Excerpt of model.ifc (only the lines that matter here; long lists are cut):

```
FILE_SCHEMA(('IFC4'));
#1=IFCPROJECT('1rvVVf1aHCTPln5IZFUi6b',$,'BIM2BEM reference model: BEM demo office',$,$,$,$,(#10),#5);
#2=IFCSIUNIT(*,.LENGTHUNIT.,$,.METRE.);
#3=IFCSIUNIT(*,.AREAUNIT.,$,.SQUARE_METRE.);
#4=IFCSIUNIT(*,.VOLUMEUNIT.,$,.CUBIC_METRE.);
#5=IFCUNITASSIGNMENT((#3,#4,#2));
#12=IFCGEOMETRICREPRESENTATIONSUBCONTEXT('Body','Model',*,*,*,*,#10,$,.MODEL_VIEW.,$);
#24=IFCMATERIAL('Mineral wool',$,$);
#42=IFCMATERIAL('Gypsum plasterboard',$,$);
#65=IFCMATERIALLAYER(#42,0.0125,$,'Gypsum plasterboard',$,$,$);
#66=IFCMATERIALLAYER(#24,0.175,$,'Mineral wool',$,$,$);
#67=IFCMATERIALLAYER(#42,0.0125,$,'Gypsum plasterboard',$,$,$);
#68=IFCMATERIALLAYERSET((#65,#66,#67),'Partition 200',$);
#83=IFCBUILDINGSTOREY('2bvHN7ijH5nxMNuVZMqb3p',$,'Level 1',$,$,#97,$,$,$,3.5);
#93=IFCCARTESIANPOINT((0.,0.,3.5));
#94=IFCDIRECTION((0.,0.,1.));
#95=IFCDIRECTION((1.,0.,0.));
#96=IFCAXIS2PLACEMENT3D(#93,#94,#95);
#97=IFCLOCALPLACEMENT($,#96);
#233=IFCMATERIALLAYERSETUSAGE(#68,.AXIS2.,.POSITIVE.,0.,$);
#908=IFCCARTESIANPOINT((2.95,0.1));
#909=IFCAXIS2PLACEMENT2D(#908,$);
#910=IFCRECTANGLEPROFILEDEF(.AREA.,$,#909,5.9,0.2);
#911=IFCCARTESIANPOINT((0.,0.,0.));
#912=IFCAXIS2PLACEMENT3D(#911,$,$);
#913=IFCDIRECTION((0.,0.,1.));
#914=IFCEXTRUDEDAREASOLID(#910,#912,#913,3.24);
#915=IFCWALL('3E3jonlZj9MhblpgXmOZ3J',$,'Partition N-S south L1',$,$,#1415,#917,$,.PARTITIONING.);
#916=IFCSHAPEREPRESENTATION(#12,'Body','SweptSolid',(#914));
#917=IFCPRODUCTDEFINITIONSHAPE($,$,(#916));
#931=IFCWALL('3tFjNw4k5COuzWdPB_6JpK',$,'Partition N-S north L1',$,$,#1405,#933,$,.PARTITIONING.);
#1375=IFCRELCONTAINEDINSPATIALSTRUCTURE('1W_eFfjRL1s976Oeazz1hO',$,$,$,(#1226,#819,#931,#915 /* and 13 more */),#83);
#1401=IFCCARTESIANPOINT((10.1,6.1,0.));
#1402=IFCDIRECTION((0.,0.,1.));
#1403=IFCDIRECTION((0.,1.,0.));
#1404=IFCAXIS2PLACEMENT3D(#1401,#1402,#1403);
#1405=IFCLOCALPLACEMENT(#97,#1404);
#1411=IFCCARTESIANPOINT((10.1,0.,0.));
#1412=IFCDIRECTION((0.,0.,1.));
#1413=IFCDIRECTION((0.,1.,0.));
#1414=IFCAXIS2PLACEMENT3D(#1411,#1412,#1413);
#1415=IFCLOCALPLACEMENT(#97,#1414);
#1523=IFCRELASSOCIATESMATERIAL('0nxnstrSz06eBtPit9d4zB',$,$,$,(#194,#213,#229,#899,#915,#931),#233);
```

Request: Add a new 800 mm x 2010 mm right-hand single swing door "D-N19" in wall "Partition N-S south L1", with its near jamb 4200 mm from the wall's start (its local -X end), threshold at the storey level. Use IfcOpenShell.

```python
import numpy as np
import ifcopenshell
import ifcopenshell.api.feature
import ifcopenshell.api.geometry
import ifcopenshell.api.root
import ifcopenshell.api.spatial
import ifcopenshell.geom
import ifcopenshell.util.element
import ifcopenshell.util.placement
import ifcopenshell.util.representation
import ifcopenshell.util.shape
import ifcopenshell.util.unit

model = ifcopenshell.open("model.ifc")
unit_scale = ifcopenshell.util.unit.calculate_unit_scale(model)
settings = ifcopenshell.geom.settings()


def volume(element):
    """Net volume in cubic metres, openings subtracted."""
    shape = ifcopenshell.geom.create_shape(settings, element)
    return ifcopenshell.util.shape.get_volume(shape.geometry)


wall = model.by_guid("3E3jonlZj9MhblpgXmOZ3J")
storey = ifcopenshell.util.element.get_container(wall, ifc_class="IfcBuildingStorey")
context = ifcopenshell.util.representation.get_context(model, "Model", "Body", "MODEL_VIEW")
before = volume(wall)

width, height, from_end, sill = 0.8, 2.01, 4.2, 0.0  # metres

# The wall runs along its own X axis, and the end named is its -X end.
wall_shape = ifcopenshell.geom.create_shape(settings, wall)
x, y, z = ifcopenshell.util.shape.get_vertices(wall_shape.geometry).T
start = x.min() + from_end
face, thickness = float(y.min()), float(y.max() - y.min())
wall_matrix = ifcopenshell.util.placement.get_local_placement(wall.ObjectPlacement)
level = ifcopenshell.util.placement.get_local_placement(storey.ObjectPlacement)[2, 3]


def in_wall(x, y):
    """Placement at x, y metres in the wall's axes, at sill height."""
    matrix = wall_matrix.copy()
    matrix[:, 3] = wall_matrix @ np.array([x / unit_scale, y / unit_scale, 0.0, 1.0])
    matrix[2, 3] = level + sill / unit_scale
    return matrix


# Opening: a box that overshoots both wall faces by 50 mm.
opening = ifcopenshell.api.root.create_entity(model, ifc_class="IfcOpeningElement", predefined_type="OPENING")
box = ifcopenshell.api.geometry.add_wall_representation(
    model, context=context, length=width, height=height, thickness=thickness + 0.1
)
ifcopenshell.api.geometry.assign_representation(model, product=opening, representation=box)
ifcopenshell.api.geometry.edit_object_placement(model, product=opening, matrix=in_wall(start, face - 0.05), is_si=False)
ifcopenshell.api.feature.add_feature(model, feature=opening, element=wall)

door = ifcopenshell.api.root.create_entity(model, ifc_class="IfcDoor", name="D-N19", predefined_type="DOOR")
door.OverallWidth, door.OverallHeight = width / unit_scale, height / unit_scale
door.OperationType = "SINGLE_SWING_RIGHT"
body = ifcopenshell.api.geometry.add_door_representation(
    model,
    context=context,
    overall_width=door.OverallWidth,
    overall_height=door.OverallHeight,
    operation_type="SINGLE_SWING_RIGHT",
    lining_properties={"LiningDepth": thickness / unit_scale, "ThresholdDepth": thickness / unit_scale},
)
ifcopenshell.api.geometry.assign_representation(model, product=door, representation=body)
ifcopenshell.api.spatial.assign_container(model, products=[door], relating_structure=storey)
ifcopenshell.api.feature.add_filling(model, opening=opening, element=door)

# The lining spans the wall, so the door starts at the wall face.
ifcopenshell.api.geometry.edit_object_placement(model, product=door, matrix=in_wall(start, face), is_si=False)

after = volume(wall)

print(f"wall volume {before:.3f} -> {after:.3f} m3")

model.write("model_updated.ifc")
```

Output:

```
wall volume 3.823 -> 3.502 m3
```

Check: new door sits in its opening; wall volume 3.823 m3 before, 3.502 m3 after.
